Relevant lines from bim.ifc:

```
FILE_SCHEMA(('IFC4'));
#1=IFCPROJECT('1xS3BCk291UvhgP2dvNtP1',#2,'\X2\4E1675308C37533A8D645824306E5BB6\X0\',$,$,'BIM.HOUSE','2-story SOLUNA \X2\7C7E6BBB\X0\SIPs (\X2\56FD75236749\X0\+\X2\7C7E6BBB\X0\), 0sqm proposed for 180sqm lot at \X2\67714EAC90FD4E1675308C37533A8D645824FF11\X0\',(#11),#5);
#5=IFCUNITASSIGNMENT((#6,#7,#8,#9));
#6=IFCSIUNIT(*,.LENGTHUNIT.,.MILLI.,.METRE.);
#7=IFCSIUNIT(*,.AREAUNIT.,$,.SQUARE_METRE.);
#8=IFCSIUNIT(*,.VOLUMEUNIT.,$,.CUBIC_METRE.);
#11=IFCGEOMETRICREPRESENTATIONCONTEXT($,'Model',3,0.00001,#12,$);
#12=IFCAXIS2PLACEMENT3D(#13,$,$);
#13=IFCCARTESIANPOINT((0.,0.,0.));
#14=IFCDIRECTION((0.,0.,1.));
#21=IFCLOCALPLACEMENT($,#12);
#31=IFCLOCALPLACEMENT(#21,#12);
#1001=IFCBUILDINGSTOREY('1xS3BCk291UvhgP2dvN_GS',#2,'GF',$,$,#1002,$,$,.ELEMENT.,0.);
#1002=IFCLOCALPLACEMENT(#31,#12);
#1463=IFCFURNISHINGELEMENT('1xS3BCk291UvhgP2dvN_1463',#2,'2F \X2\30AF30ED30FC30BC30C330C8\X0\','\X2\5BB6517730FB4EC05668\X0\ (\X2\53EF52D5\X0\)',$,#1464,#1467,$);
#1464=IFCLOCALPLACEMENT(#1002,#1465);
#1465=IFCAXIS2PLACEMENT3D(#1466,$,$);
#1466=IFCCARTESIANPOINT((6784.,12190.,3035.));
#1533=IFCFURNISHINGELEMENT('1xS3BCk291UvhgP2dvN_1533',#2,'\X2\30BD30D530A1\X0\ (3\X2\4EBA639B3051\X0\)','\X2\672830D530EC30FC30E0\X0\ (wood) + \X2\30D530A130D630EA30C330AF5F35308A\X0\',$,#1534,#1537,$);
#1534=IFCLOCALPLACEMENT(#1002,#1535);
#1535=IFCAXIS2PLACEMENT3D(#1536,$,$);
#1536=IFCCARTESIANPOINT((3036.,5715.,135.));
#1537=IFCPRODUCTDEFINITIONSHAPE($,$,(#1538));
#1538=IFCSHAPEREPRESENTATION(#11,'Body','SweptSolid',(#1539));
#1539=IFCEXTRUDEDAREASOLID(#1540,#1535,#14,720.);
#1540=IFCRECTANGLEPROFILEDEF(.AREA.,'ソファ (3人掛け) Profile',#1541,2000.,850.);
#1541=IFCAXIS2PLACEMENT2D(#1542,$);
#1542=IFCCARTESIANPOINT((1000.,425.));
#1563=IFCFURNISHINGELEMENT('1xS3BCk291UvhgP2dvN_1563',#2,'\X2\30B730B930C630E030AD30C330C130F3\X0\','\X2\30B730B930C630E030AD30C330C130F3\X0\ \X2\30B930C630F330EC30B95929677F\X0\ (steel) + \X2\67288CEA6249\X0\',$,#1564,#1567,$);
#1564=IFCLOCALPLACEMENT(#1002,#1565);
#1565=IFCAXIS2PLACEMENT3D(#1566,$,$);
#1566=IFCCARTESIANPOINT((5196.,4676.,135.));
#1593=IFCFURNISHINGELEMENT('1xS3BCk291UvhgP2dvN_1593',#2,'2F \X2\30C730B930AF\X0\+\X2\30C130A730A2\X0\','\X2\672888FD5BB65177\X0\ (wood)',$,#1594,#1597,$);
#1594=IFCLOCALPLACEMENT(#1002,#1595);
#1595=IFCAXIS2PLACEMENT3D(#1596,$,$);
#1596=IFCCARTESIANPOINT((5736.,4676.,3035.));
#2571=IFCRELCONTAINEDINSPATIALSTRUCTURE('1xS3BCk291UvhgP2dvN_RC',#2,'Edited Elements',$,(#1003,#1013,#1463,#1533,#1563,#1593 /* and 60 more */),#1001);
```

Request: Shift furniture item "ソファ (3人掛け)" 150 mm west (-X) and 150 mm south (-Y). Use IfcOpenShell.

```python
import ifcopenshell
import ifcopenshell.api.geometry
import ifcopenshell.util.placement

model = ifcopenshell.open("bim.ifc")

item = model.by_guid("1xS3BCk291UvhgP2dvN_1533")
matrix = ifcopenshell.util.placement.get_local_placement(item.ObjectPlacement)
matrix[0, 3] -= 150.0
matrix[1, 3] -= 150.0
ifcopenshell.api.geometry.edit_object_placement(model, product=item, matrix=matrix, is_si=False)

print(ifcopenshell.util.placement.get_local_placement(item.ObjectPlacement).round(3) + 0.0)

model.write("bim_updated.ifc")
```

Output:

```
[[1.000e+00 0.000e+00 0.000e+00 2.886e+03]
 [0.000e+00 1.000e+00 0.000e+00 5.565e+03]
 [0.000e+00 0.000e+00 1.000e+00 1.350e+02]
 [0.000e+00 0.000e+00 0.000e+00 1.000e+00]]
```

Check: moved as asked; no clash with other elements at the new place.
